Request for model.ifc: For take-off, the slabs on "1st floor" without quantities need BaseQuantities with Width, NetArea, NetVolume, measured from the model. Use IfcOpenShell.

First a look at what the model holds.

```python
import ifcopenshell
import ifcopenshell.util.element
import ifcopenshell.util.unit

model = ifcopenshell.open("model.ifc")
print(model.schema)
for unit_type in ("LENGTHUNIT", "AREAUNIT", "VOLUMEUNIT"):
    print(unit_type, ifcopenshell.util.unit.calculate_unit_scale(model, unit_type))
storey = next(s for s in model.by_type("IfcBuildingStorey") if s.Name == "1st floor")
slabs = [e for e in ifcopenshell.util.element.get_decomposition(storey) if e.is_a("IfcSlab")]
for e in sorted(slabs, key=lambda e: e.id()):
    print(e.id(), e.is_a(), e.Name, list(ifcopenshell.util.element.get_psets(e, qtos_only=True)), sep=" | ")
```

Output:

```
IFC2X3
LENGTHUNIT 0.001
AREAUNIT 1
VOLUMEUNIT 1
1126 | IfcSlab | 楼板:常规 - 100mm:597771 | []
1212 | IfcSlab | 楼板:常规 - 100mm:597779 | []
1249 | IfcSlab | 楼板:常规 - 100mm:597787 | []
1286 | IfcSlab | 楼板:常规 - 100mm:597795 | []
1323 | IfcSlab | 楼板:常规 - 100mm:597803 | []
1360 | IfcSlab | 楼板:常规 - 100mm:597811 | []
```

```python
import ifcopenshell
import ifcopenshell.api.pset
import ifcopenshell.geom
import ifcopenshell.util.element
import ifcopenshell.util.shape
import ifcopenshell.util.unit

model = ifcopenshell.open("model.ifc")
unit_scale = ifcopenshell.util.unit.calculate_unit_scale(model)
area_scale = ifcopenshell.util.unit.calculate_unit_scale(model, "AREAUNIT")
volume_scale = ifcopenshell.util.unit.calculate_unit_scale(model, "VOLUMEUNIT")
settings = ifcopenshell.geom.settings()

storey = next(s for s in model.by_type("IfcBuildingStorey") if s.Name == "1st floor")
slabs = [e for e in ifcopenshell.util.element.get_decomposition(storey) if e.is_a("IfcSlab")]

for e in sorted(slabs, key=lambda e: e.id()):
    if ifcopenshell.util.element.get_psets(e, qtos_only=True, should_inherit=False):
        continue
    # Geometry comes back in metres, in the element's own axes.
    shape = ifcopenshell.geom.create_shape(settings, e)
    values = {
        "Width": ifcopenshell.util.shape.get_z(shape.geometry) / unit_scale,
        "NetArea": ifcopenshell.util.shape.get_footprint_area(shape.geometry) / area_scale,
        "NetVolume": ifcopenshell.util.shape.get_volume(shape.geometry) / volume_scale,
    }
    qto = ifcopenshell.api.pset.add_qto(model, product=e, name="BaseQuantities")
    ifcopenshell.api.pset.edit_qto(model, qto=qto, properties=values)
    print(e.id(), {k: round(v, 3) for k, v in values.items()})

model.write("model_edited.ifc")
```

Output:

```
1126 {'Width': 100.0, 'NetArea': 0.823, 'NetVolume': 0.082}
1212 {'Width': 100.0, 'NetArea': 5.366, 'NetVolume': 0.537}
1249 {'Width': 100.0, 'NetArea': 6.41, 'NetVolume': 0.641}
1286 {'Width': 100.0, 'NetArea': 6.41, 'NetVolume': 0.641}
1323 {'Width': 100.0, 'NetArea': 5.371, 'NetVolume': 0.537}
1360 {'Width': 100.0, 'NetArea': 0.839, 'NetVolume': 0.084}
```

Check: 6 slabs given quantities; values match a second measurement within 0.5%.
